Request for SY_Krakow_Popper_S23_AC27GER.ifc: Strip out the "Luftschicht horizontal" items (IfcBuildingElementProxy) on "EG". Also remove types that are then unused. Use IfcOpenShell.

First a look at what the model holds.

```python
import ifcopenshell
import ifcopenshell.util.element

model = ifcopenshell.open("SY_Krakow_Popper_S23_AC27GER.ifc")
print(model.schema)
storey = next(s for s in model.by_type("IfcBuildingStorey") if s.Name == "EG")
proxies = [e for e in ifcopenshell.util.element.get_decomposition(storey) if e.is_a("IfcBuildingElementProxy")]
seen = {}
for e in proxies:
    element_type = ifcopenshell.util.element.get_type(e)
    name = element_type.Name if element_type not in (None, e) else None
    seen[name] = seen.get(name, 0) + 1
for name, count in sorted(seen.items(), key=str):
    print(count, "x", name)
```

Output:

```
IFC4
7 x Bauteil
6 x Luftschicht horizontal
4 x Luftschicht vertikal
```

```python
import ifcopenshell
import ifcopenshell.api.root
import ifcopenshell.util.element

model = ifcopenshell.open("SY_Krakow_Popper_S23_AC27GER.ifc")

storey = next(s for s in model.by_type("IfcBuildingStorey") if s.Name == "EG")
proxies = [e for e in ifcopenshell.util.element.get_decomposition(storey) if e.is_a("IfcBuildingElementProxy")]
targets = [e for e in proxies if (t := ifcopenshell.util.element.get_type(e)) not in (None, e) and t.Name == "Luftschicht horizontal"]
types = {ifcopenshell.util.element.get_type(e) for e in targets} - {None, *targets}

for e in targets:
    ifcopenshell.api.root.remove_product(model, product=e)
print(len(targets), "removed")

unused = [t for t in types if not ifcopenshell.util.element.get_types(t)]
for t in unused:
    ifcopenshell.api.root.remove_product(model, product=t)
print(len(unused), "unused types removed")

model.write("SY_Krakow_Popper_S23_AC27GER_v2.ifc")
```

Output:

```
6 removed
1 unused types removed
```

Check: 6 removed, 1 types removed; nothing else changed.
